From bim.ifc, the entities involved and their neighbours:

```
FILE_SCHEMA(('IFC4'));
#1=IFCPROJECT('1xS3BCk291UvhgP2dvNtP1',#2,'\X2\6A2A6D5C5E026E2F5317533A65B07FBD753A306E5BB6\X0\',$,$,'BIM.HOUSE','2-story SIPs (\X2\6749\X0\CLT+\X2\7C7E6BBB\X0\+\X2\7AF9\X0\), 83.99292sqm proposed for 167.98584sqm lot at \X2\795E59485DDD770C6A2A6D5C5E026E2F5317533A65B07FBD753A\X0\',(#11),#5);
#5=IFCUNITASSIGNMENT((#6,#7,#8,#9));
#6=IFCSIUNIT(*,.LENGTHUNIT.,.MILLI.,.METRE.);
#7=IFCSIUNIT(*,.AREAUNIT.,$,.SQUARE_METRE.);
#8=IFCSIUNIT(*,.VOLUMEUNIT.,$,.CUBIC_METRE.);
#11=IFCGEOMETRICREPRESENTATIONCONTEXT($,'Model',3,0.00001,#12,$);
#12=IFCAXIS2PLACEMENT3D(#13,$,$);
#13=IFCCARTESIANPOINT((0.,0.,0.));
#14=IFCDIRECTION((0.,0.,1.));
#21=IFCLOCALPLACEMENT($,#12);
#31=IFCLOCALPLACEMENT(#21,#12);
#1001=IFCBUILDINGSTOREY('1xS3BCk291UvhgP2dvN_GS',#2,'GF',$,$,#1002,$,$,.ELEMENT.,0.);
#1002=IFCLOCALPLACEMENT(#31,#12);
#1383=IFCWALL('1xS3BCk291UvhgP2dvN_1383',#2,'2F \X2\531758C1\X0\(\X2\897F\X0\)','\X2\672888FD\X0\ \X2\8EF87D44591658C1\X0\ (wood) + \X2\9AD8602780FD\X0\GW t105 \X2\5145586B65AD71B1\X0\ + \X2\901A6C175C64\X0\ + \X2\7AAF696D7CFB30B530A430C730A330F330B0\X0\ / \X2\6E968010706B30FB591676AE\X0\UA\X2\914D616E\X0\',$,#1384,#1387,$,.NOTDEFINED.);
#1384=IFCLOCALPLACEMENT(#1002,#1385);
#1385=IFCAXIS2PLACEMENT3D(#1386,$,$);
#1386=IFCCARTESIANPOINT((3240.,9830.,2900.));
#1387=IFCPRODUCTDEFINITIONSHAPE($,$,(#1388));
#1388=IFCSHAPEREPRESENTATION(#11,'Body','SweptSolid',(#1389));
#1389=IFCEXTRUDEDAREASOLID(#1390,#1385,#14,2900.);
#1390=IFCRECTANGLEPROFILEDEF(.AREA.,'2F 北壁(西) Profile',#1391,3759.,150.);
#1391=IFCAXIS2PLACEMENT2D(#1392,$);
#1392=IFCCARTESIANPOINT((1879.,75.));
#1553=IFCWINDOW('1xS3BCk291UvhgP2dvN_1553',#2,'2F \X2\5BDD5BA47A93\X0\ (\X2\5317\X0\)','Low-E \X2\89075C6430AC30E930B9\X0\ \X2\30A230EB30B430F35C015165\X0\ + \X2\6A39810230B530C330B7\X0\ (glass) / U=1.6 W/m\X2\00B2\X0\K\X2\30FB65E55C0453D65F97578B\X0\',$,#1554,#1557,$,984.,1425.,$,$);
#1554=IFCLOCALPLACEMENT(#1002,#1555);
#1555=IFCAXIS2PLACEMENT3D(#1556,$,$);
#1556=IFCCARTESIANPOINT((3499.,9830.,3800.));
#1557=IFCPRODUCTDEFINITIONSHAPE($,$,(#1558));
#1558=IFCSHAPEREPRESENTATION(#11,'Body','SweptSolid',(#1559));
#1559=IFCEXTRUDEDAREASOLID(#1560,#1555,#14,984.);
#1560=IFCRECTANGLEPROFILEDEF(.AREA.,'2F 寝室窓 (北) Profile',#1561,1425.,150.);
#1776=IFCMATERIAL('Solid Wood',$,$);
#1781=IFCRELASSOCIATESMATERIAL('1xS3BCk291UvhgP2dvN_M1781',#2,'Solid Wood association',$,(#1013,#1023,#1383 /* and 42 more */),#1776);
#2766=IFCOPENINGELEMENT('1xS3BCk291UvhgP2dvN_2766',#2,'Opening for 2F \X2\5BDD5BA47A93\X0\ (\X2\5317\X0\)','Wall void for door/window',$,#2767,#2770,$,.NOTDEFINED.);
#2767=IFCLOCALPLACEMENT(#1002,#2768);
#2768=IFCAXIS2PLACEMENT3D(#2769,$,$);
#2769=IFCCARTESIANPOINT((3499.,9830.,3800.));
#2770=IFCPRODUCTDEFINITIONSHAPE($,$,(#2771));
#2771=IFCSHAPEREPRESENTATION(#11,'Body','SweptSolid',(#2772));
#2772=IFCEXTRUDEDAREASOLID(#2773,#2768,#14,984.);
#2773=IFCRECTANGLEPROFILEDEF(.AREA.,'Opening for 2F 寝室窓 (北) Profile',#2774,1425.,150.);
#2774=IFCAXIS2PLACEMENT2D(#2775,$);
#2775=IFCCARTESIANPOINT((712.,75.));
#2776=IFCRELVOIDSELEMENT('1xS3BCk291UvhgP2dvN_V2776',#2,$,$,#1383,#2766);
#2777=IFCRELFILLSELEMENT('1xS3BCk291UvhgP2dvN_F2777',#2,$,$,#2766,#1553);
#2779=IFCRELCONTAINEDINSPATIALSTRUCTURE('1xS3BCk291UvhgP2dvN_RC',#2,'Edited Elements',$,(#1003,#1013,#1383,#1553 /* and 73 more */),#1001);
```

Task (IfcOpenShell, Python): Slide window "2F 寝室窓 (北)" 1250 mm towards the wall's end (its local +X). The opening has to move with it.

```python
import ifcopenshell
import ifcopenshell.api.geometry
import ifcopenshell.util.placement
import ifcopenshell.util.unit

model = ifcopenshell.open("bim.ifc")
unit_scale = ifcopenshell.util.unit.calculate_unit_scale(model)

window = model.by_id(1553)
opening = window.FillsVoids[0].RelatingOpeningElement
wall = opening.VoidsElements[0].RelatingBuildingElement

wall_matrix = ifcopenshell.util.placement.get_local_placement(wall.ObjectPlacement)
shift = wall_matrix[:3, 0] * 1.25 / unit_scale
before = ifcopenshell.util.placement.get_local_placement(window.ObjectPlacement)[:3, 3].copy()

# The window is not placed relative to its opening, so move both.
for product in (opening, window):
    matrix = ifcopenshell.util.placement.get_local_placement(product.ObjectPlacement)
    matrix[:3, 3] += shift
    ifcopenshell.api.geometry.edit_object_placement(model, product=product, matrix=matrix, is_si=False)

after = ifcopenshell.util.placement.get_local_placement(window.ObjectPlacement)[:3, 3]
print("window moved by", (after - before).round(3) + 0.0)

model.write("bim_v2.ifc")
```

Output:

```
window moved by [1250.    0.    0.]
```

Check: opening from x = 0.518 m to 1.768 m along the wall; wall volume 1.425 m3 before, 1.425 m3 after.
